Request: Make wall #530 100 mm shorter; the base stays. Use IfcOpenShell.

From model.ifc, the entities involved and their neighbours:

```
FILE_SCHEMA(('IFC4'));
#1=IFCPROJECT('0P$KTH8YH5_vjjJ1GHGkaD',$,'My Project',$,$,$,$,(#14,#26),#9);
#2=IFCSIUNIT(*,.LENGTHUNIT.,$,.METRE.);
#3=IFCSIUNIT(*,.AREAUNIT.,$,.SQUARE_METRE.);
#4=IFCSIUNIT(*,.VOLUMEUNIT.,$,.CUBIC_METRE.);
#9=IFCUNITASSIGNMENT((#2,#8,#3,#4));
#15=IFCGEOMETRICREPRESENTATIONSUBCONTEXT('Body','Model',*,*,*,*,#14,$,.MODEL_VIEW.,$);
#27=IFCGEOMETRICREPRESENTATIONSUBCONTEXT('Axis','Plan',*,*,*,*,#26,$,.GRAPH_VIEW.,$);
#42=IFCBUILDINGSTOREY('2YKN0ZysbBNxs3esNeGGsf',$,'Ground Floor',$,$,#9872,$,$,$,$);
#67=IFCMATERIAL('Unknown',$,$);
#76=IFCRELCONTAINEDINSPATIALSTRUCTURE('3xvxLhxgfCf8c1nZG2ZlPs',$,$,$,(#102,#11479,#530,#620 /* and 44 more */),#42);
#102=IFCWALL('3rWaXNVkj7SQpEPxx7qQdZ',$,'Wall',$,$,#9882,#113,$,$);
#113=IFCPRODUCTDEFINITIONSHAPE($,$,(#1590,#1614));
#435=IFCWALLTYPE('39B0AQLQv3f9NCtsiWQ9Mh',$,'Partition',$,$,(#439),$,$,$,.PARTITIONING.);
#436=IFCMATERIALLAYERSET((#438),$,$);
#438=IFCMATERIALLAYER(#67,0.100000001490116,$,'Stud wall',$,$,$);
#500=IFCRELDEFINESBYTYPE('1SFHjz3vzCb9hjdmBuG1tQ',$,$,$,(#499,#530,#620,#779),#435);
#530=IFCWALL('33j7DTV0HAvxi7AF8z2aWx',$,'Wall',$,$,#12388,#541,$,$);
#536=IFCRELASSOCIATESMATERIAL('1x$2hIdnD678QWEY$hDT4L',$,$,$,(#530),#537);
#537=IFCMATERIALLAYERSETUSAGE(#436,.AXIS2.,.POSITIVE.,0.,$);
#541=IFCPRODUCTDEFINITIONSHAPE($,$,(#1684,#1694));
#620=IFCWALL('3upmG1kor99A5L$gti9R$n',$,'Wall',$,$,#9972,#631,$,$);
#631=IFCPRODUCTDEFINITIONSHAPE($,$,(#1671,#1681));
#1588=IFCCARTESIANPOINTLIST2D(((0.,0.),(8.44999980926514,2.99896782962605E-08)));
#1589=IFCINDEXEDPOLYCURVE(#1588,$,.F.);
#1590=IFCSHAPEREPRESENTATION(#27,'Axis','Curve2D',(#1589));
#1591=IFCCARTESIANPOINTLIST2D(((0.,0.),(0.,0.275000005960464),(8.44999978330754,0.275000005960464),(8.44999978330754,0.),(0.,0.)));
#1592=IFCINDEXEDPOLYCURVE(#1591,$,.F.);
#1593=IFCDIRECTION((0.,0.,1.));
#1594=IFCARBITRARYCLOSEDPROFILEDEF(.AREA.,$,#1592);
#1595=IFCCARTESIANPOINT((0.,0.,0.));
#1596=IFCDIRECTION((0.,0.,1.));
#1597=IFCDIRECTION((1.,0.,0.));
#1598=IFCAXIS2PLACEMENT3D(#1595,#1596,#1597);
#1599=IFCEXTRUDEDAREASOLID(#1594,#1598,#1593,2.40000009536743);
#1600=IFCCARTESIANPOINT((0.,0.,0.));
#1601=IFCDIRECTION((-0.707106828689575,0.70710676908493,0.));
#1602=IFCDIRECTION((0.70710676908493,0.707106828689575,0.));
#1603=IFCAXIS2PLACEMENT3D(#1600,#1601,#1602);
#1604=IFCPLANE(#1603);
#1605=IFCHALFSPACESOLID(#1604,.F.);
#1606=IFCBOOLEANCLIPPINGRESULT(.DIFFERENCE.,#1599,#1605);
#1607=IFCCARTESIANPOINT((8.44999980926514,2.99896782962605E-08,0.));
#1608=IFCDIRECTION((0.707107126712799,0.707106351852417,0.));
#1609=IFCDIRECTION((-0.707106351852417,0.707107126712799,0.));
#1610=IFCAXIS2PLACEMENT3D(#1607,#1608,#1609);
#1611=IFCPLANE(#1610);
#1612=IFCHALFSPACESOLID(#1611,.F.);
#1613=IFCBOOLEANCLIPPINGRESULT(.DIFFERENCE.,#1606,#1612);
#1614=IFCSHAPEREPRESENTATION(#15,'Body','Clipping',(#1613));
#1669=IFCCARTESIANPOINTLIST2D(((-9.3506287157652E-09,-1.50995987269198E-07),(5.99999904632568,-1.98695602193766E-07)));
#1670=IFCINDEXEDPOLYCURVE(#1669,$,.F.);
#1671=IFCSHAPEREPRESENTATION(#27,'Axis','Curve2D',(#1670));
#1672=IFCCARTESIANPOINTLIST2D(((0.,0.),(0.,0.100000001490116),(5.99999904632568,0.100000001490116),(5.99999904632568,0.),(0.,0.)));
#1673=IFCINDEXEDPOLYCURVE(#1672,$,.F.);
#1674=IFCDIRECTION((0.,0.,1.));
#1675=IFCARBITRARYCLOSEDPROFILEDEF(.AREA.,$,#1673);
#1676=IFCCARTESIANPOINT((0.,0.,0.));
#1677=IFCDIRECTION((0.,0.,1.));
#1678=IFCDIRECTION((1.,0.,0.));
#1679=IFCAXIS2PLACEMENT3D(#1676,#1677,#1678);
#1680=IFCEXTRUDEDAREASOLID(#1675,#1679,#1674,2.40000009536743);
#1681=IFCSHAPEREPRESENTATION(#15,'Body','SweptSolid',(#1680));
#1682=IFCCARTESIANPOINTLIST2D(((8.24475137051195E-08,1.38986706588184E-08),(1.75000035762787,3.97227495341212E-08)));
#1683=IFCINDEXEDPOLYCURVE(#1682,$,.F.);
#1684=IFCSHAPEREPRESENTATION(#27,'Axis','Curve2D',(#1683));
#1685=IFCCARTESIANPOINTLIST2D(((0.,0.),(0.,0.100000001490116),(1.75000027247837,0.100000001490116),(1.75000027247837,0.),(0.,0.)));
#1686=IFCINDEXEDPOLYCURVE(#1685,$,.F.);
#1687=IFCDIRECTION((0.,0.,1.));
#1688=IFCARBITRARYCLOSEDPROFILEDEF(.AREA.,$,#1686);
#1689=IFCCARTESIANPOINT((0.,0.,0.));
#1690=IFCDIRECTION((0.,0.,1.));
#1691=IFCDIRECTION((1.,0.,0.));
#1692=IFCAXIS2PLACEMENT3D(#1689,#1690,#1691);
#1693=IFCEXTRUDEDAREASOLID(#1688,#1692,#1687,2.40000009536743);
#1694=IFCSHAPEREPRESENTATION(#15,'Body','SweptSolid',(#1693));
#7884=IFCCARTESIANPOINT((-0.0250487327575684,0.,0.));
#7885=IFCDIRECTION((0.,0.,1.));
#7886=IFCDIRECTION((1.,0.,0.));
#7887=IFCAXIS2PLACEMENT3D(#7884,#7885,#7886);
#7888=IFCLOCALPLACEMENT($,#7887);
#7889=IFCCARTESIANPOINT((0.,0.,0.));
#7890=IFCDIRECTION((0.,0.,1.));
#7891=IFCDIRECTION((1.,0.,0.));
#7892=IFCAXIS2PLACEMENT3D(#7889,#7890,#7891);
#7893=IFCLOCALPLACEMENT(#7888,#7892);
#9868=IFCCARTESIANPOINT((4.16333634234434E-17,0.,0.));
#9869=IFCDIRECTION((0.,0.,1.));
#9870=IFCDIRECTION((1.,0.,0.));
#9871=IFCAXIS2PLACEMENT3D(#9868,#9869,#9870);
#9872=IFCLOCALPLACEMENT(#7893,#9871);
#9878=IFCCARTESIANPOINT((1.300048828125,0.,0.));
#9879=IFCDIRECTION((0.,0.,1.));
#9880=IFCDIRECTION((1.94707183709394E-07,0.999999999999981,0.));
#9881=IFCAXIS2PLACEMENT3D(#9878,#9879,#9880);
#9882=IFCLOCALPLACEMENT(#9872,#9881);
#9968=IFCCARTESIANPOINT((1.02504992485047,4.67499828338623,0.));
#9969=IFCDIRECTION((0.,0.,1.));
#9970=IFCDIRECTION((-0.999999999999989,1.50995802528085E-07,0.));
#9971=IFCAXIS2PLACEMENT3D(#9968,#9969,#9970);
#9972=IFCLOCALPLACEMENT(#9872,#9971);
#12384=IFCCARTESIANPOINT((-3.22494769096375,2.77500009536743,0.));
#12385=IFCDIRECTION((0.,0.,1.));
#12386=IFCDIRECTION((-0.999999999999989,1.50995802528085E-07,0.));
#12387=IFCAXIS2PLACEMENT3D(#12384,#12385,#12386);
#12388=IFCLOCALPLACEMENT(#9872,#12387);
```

```python
import ifcopenshell
import ifcopenshell.geom
import ifcopenshell.util.representation
import ifcopenshell.util.shape

model = ifcopenshell.open("model.ifc")
settings = ifcopenshell.geom.settings()


def volume(element):
    """Net volume in cubic metres, openings subtracted."""
    shape = ifcopenshell.geom.create_shape(settings, element)
    return ifcopenshell.util.shape.get_volume(shape.geometry)


wall = model.by_id(530)
before = volume(wall)

body = ifcopenshell.util.representation.get_representation(wall, "Model", "Body")
solid = body.Items[0]
old_height = solid.Depth
solid.Depth -= 0.1
after = volume(wall)

print(f"height {old_height:g} -> {solid.Depth:g}, volume {before:.3f} -> {after:.3f} m3")

model.write("model_edited.ifc")
```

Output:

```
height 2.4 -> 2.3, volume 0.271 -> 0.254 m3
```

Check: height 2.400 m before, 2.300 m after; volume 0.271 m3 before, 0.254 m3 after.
